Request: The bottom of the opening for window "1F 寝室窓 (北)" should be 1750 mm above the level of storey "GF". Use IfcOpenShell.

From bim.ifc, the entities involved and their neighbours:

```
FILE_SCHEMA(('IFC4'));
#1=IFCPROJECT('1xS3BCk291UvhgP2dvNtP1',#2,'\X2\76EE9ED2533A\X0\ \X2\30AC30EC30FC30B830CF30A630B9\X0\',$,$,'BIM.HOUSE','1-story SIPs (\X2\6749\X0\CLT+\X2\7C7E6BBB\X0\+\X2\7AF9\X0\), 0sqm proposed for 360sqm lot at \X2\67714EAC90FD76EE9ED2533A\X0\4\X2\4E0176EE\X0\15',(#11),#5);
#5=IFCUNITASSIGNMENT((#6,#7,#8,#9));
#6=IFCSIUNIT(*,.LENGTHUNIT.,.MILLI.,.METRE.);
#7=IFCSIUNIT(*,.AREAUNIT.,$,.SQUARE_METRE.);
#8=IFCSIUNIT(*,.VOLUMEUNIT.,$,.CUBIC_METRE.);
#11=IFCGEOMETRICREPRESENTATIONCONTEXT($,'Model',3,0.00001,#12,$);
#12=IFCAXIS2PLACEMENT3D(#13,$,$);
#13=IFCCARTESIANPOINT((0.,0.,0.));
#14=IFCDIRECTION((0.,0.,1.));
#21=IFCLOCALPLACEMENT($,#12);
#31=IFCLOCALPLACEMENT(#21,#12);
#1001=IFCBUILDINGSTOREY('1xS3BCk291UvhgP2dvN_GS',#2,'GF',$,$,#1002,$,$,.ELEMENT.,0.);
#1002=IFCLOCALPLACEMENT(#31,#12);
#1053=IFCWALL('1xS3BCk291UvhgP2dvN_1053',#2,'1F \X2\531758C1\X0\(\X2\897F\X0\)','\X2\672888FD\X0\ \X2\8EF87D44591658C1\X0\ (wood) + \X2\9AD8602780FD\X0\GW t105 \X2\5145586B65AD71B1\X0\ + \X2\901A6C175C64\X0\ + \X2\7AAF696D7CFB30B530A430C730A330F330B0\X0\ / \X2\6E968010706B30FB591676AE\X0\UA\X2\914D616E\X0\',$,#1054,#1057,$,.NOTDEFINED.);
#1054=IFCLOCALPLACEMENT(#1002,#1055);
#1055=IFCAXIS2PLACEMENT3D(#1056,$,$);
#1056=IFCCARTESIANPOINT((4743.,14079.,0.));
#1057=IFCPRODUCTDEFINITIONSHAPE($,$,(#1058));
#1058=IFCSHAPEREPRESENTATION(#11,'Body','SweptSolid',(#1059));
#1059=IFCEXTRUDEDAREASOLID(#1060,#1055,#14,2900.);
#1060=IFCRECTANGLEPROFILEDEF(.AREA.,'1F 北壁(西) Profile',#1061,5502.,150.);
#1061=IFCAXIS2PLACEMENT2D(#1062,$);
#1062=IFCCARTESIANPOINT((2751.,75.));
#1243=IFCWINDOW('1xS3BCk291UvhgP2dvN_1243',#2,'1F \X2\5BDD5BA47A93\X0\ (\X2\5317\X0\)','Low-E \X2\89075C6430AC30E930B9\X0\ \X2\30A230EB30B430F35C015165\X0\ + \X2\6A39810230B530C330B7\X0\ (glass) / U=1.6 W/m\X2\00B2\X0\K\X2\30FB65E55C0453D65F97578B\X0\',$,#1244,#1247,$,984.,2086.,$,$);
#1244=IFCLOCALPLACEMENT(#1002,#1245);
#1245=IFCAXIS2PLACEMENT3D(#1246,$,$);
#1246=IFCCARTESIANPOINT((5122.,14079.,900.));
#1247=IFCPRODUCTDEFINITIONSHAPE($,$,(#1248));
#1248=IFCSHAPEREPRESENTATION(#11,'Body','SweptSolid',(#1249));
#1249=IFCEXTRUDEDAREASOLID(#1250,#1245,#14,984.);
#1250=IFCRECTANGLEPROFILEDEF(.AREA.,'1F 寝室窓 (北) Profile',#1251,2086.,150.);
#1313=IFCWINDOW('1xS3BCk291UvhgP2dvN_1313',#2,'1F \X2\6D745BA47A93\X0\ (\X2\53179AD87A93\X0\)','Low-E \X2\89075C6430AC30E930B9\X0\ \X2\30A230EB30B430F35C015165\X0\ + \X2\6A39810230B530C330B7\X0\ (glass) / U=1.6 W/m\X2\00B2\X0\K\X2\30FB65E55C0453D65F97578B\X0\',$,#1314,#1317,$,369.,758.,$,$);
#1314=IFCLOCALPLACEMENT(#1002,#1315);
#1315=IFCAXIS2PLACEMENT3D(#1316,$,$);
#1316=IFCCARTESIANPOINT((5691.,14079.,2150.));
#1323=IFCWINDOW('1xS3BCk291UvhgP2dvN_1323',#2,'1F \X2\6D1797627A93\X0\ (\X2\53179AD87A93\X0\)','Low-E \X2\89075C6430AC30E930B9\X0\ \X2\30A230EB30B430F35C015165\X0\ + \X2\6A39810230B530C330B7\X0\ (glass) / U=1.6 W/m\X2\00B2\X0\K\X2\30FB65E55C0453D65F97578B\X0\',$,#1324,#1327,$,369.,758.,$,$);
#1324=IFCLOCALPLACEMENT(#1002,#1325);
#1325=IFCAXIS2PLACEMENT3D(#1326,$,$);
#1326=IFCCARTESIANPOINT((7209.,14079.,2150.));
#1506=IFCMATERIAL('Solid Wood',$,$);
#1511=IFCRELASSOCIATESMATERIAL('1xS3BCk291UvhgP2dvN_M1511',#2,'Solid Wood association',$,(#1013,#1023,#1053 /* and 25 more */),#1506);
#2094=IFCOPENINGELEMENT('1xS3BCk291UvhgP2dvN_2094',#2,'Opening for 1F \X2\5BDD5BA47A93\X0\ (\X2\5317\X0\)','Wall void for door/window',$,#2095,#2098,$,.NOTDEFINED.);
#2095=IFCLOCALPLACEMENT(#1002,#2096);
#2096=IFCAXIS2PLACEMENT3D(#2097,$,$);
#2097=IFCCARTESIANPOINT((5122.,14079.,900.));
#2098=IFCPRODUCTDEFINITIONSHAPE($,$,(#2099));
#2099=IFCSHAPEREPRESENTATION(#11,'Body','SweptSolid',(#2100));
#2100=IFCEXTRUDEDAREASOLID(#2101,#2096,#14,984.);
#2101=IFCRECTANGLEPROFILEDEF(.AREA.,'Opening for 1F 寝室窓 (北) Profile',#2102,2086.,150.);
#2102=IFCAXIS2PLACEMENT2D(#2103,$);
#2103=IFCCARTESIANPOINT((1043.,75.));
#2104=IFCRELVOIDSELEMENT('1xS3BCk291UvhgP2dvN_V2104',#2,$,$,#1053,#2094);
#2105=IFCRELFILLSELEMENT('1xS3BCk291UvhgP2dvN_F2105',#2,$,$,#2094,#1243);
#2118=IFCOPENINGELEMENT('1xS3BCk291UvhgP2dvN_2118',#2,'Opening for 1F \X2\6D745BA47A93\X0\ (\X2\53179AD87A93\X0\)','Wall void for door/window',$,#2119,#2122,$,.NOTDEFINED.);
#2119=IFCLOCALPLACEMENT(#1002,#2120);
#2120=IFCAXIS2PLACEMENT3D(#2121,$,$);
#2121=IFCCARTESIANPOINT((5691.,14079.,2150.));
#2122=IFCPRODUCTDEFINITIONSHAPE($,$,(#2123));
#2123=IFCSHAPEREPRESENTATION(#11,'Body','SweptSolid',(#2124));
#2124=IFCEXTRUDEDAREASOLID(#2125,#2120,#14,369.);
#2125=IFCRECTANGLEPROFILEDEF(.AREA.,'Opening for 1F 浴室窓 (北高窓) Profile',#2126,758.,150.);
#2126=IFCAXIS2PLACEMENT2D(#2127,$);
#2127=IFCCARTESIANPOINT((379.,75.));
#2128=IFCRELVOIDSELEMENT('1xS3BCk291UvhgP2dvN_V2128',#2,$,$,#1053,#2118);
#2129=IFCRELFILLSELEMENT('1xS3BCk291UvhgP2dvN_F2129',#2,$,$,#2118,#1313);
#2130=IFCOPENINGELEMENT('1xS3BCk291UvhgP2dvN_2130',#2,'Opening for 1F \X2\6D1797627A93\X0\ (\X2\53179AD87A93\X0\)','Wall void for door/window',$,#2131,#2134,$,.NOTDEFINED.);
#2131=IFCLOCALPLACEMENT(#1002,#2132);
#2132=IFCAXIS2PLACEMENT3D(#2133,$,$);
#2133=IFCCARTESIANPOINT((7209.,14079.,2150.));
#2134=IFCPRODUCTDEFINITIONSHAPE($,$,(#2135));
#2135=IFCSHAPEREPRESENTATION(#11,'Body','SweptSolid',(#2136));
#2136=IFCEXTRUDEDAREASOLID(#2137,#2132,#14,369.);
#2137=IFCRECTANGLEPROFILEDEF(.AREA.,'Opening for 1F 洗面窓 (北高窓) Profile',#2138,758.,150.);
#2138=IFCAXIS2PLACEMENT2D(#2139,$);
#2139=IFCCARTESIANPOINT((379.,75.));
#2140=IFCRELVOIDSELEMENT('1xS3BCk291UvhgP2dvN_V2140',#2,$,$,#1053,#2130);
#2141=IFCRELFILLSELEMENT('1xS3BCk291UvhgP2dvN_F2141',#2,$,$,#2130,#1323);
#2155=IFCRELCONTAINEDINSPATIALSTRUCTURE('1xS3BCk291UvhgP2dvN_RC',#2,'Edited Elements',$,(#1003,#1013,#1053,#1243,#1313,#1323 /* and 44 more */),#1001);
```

```python
import numpy as np
import ifcopenshell
import ifcopenshell.api.geometry
import ifcopenshell.geom
import ifcopenshell.util.element
import ifcopenshell.util.placement
import ifcopenshell.util.shape
import ifcopenshell.util.unit

model = ifcopenshell.open("bim.ifc")
unit_scale = ifcopenshell.util.unit.calculate_unit_scale(model)

window = model.by_id(1243)
opening = window.FillsVoids[0].RelatingOpeningElement
storey = ifcopenshell.util.element.get_container(window, ifc_class="IfcBuildingStorey")
level = ifcopenshell.util.placement.get_local_placement(storey.ObjectPlacement)[2, 3]

# The opening's origin need not be at the sill, so measure its lowest point.
shape = ifcopenshell.geom.create_shape(ifcopenshell.geom.settings(), opening)
bottom = ifcopenshell.util.shape.get_shape_bottom_elevation(shape, shape.geometry) / unit_scale
dz = level + 1750.0 - bottom

shift = np.array([0.0, 0.0, dz])
# The window is not placed relative to its opening, so move both.
for product in (opening, window):
    matrix = ifcopenshell.util.placement.get_local_placement(product.ObjectPlacement)
    matrix[:3, 3] += shift
    ifcopenshell.api.geometry.edit_object_placement(model, product=product, matrix=matrix, is_si=False)

print(f"moved by {dz * unit_scale:+.3f} m")

model.write("bim-out.ifc")
```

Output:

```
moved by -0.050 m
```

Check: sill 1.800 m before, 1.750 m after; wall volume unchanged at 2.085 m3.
